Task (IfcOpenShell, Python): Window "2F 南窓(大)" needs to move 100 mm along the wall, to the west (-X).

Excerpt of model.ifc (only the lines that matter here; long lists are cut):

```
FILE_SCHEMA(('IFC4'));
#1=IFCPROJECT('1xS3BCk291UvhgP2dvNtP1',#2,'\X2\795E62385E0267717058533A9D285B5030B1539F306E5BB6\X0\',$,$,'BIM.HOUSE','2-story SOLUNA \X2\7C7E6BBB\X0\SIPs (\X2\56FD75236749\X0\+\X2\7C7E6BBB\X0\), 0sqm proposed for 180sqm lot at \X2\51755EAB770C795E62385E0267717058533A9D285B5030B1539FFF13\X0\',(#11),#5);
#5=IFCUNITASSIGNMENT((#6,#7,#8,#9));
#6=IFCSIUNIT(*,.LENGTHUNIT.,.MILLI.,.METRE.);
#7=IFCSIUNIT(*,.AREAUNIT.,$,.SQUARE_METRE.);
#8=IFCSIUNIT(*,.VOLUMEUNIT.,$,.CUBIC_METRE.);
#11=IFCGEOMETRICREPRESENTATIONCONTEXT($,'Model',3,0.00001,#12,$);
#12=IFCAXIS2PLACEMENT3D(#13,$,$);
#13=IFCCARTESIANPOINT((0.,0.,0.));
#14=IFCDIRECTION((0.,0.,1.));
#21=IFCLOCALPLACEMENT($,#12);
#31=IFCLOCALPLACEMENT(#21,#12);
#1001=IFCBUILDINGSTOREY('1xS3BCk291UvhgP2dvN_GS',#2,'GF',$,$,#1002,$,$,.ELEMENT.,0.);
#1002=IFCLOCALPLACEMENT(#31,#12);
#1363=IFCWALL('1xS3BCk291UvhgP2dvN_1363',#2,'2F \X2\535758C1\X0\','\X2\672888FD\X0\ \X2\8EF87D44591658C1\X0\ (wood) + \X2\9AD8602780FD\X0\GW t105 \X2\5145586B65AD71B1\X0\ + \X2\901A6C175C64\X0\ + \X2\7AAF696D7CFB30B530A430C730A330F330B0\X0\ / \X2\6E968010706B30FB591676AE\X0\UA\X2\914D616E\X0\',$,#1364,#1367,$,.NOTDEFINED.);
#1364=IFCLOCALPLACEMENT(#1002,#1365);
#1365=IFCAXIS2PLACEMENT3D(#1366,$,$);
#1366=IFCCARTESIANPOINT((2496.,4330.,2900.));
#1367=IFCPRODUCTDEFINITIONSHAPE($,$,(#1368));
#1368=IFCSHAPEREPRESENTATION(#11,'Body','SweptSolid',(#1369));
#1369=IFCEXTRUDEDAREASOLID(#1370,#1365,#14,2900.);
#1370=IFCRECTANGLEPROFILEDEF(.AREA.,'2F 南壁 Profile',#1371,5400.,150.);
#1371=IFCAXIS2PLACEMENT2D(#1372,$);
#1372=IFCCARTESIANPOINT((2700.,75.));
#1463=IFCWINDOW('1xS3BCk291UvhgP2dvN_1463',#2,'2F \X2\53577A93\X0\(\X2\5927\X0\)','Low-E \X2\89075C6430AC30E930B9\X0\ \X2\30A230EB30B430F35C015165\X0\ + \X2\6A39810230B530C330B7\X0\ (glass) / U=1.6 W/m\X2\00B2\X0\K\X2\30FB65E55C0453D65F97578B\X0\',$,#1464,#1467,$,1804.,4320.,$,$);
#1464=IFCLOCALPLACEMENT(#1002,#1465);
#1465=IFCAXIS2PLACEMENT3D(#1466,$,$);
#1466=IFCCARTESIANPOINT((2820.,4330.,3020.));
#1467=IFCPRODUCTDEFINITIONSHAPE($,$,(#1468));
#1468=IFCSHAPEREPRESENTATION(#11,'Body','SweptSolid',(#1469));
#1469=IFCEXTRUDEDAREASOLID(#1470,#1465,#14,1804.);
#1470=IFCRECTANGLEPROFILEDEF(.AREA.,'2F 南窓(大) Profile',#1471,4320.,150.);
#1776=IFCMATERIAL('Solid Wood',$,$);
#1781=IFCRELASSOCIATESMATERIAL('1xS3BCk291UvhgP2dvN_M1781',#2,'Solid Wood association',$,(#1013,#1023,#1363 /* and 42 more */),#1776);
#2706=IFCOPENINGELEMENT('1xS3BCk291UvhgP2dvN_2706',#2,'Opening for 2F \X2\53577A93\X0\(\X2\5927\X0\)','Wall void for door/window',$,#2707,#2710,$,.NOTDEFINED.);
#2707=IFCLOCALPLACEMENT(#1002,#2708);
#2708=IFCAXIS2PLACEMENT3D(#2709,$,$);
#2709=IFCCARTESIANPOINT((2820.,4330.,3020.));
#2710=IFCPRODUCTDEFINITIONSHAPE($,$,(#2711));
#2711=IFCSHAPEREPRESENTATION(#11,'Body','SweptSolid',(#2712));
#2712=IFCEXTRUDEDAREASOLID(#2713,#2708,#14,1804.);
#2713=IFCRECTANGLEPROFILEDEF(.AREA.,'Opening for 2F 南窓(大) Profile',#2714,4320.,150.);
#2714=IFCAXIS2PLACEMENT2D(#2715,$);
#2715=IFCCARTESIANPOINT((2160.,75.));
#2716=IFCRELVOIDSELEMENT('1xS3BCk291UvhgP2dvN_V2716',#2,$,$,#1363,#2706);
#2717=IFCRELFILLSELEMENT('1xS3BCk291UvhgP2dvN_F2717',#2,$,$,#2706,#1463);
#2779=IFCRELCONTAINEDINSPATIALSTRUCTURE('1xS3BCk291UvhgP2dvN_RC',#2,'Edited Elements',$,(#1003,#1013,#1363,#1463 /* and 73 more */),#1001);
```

```python
import ifcopenshell
import ifcopenshell.api.geometry
import ifcopenshell.util.placement

model = ifcopenshell.open("model.ifc")

window = model.by_guid("1xS3BCk291UvhgP2dvN_1463")
opening = window.FillsVoids[0].RelatingOpeningElement
wall = opening.VoidsElements[0].RelatingBuildingElement

wall_matrix = ifcopenshell.util.placement.get_local_placement(wall.ObjectPlacement)
shift = wall_matrix[:3, 0] * -100.0
before = ifcopenshell.util.placement.get_local_placement(window.ObjectPlacement)[:3, 3].copy()

# The window is not placed relative to its opening, so move both.
for product in (opening, window):
    matrix = ifcopenshell.util.placement.get_local_placement(product.ObjectPlacement)
    matrix[:3, 3] += shift
    ifcopenshell.api.geometry.edit_object_placement(model, product=product, matrix=matrix, is_si=False)

after = ifcopenshell.util.placement.get_local_placement(window.ObjectPlacement)[:3, 3]
print("window moved by", (after - before).round(3) + 0.0)

model.write("model-out.ifc")
```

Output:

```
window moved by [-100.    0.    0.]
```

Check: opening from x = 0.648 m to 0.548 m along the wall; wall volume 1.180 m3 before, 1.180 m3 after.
